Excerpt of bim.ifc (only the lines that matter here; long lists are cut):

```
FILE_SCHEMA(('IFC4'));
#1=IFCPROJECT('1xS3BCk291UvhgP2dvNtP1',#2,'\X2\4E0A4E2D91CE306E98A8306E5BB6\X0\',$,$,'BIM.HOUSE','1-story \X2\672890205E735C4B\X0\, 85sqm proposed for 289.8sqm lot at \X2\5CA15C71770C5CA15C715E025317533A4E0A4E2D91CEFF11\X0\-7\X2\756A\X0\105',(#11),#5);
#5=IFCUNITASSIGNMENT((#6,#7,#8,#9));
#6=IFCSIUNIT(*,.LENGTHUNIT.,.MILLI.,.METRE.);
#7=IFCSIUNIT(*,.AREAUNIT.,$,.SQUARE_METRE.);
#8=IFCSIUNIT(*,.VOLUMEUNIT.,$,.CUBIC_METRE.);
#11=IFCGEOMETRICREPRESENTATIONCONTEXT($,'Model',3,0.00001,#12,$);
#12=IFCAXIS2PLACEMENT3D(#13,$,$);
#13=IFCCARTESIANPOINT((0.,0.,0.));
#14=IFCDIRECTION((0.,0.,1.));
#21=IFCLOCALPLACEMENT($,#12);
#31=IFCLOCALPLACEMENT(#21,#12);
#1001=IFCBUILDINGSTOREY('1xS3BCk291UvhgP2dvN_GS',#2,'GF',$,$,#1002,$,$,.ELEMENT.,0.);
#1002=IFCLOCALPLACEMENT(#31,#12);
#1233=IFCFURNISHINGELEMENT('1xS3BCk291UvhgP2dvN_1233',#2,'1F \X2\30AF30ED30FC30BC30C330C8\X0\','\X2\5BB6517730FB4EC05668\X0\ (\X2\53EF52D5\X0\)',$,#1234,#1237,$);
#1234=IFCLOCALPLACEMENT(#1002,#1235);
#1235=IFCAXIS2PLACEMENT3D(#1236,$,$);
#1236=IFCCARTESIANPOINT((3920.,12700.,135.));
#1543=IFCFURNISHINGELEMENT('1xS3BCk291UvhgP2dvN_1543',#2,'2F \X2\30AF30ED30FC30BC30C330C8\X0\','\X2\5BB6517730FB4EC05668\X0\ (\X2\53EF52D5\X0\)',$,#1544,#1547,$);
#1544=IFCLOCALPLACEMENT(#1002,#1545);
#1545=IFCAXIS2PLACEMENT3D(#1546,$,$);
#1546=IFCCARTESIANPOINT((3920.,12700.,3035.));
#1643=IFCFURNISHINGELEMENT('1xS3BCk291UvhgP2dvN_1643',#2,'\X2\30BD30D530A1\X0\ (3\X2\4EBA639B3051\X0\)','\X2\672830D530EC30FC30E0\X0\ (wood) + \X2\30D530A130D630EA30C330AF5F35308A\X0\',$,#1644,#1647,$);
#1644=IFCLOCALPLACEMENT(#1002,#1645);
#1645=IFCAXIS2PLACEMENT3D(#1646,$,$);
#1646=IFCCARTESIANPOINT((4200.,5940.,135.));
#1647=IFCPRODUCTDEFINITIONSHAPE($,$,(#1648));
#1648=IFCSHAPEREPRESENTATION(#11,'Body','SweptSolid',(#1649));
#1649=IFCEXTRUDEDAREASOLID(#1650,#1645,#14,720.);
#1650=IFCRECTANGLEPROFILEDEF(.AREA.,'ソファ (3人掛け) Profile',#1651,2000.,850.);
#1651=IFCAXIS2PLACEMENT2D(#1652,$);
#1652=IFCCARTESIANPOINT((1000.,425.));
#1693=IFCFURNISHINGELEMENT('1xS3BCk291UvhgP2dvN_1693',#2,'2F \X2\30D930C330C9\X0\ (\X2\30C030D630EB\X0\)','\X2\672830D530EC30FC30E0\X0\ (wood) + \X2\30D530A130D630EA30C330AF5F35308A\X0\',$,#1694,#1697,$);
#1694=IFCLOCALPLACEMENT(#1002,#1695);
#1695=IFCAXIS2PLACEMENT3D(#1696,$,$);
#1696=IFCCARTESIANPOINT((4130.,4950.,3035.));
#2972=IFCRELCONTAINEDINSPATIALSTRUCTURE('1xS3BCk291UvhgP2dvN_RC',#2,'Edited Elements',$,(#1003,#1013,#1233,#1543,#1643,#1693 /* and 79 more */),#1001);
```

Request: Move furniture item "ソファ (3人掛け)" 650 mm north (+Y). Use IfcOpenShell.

```python
import ifcopenshell
import ifcopenshell.api.geometry
import ifcopenshell.util.placement

model = ifcopenshell.open("bim.ifc")

item = model.by_guid("1xS3BCk291UvhgP2dvN_1643")
matrix = ifcopenshell.util.placement.get_local_placement(item.ObjectPlacement)
matrix[1, 3] += 650.0
ifcopenshell.api.geometry.edit_object_placement(model, product=item, matrix=matrix, is_si=False)

print(ifcopenshell.util.placement.get_local_placement(item.ObjectPlacement).round(3) + 0.0)

model.write("bim-out.ifc")
```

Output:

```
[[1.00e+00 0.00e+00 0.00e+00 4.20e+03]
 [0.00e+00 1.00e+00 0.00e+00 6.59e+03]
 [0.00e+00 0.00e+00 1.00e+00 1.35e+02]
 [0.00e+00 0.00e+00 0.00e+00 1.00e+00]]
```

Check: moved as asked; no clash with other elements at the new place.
